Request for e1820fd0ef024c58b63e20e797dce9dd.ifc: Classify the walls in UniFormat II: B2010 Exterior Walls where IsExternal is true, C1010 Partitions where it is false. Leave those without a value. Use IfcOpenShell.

First a look at what the model holds.

```python
import ifcopenshell
import ifcopenshell.util.element

model = ifcopenshell.open("e1820fd0ef024c58b63e20e797dce9dd.ifc")
print(model.schema)
print("classifications:", [c.Name for c in model.by_type("IfcClassification")])
values = [ifcopenshell.util.element.get_pset(e, "Pset_WallCommon", "IsExternal") for e in model.by_type("IfcWall")]
for value in (True, False, None):
    print("IsExternal", value, values.count(value))
```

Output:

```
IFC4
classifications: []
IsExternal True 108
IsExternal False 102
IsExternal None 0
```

```python
import ifcopenshell
import ifcopenshell.api.classification
import ifcopenshell.util.element

model = ifcopenshell.open("e1820fd0ef024c58b63e20e797dce9dd.ifc")

system = ifcopenshell.api.classification.add_classification(model, classification="UniFormat II")

walls = model.by_type("IfcWall")
external = {e: ifcopenshell.util.element.get_pset(e, "Pset_WallCommon", "IsExternal") for e in walls}
for flag, code, name in ((True, "B2010", "Exterior Walls"), (False, "C1010", "Partitions")):
    products = [e for e in walls if external[e] is flag]
    ifcopenshell.api.classification.add_reference(
        model, products=products, classification=system, identification=code, name=name
    )
    print(code, len(products))

model.write("e1820fd0ef024c58b63e20e797dce9dd_rev.ifc")
```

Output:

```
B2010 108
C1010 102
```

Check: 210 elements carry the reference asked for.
